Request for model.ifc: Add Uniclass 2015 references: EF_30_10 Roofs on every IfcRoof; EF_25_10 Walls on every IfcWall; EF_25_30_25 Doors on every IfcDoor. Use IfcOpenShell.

First a look at what the model holds.

```python
import ifcopenshell

model = ifcopenshell.open("model.ifc")
print(model.schema)
print("classifications:", [c.Name for c in model.by_type("IfcClassification")])
for ifc_class in ("IfcDoor", "IfcRoof", "IfcStair", "IfcWall", "IfcWindow"):
    print(ifc_class, len(model.by_type(ifc_class)))
```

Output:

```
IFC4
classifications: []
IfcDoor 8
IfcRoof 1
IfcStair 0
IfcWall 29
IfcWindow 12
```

```python
import ifcopenshell
import ifcopenshell.api.classification

model = ifcopenshell.open("model.ifc")

system = ifcopenshell.api.classification.add_classification(model, classification="Uniclass 2015")

codes = {
    "IfcRoof": ("EF_30_10", "Roofs"),
    "IfcWall": ("EF_25_10", "Walls"),
    "IfcDoor": ("EF_25_30_25", "Doors"),
}
for ifc_class, (code, name) in codes.items():
    products = model.by_type(ifc_class)
    ifcopenshell.api.classification.add_reference(
        model, products=products, classification=system, identification=code, name=name
    )
    print(code, len(products))

model.write("model_edited.ifc")
```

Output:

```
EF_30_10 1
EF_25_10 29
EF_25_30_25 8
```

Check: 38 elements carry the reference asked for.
